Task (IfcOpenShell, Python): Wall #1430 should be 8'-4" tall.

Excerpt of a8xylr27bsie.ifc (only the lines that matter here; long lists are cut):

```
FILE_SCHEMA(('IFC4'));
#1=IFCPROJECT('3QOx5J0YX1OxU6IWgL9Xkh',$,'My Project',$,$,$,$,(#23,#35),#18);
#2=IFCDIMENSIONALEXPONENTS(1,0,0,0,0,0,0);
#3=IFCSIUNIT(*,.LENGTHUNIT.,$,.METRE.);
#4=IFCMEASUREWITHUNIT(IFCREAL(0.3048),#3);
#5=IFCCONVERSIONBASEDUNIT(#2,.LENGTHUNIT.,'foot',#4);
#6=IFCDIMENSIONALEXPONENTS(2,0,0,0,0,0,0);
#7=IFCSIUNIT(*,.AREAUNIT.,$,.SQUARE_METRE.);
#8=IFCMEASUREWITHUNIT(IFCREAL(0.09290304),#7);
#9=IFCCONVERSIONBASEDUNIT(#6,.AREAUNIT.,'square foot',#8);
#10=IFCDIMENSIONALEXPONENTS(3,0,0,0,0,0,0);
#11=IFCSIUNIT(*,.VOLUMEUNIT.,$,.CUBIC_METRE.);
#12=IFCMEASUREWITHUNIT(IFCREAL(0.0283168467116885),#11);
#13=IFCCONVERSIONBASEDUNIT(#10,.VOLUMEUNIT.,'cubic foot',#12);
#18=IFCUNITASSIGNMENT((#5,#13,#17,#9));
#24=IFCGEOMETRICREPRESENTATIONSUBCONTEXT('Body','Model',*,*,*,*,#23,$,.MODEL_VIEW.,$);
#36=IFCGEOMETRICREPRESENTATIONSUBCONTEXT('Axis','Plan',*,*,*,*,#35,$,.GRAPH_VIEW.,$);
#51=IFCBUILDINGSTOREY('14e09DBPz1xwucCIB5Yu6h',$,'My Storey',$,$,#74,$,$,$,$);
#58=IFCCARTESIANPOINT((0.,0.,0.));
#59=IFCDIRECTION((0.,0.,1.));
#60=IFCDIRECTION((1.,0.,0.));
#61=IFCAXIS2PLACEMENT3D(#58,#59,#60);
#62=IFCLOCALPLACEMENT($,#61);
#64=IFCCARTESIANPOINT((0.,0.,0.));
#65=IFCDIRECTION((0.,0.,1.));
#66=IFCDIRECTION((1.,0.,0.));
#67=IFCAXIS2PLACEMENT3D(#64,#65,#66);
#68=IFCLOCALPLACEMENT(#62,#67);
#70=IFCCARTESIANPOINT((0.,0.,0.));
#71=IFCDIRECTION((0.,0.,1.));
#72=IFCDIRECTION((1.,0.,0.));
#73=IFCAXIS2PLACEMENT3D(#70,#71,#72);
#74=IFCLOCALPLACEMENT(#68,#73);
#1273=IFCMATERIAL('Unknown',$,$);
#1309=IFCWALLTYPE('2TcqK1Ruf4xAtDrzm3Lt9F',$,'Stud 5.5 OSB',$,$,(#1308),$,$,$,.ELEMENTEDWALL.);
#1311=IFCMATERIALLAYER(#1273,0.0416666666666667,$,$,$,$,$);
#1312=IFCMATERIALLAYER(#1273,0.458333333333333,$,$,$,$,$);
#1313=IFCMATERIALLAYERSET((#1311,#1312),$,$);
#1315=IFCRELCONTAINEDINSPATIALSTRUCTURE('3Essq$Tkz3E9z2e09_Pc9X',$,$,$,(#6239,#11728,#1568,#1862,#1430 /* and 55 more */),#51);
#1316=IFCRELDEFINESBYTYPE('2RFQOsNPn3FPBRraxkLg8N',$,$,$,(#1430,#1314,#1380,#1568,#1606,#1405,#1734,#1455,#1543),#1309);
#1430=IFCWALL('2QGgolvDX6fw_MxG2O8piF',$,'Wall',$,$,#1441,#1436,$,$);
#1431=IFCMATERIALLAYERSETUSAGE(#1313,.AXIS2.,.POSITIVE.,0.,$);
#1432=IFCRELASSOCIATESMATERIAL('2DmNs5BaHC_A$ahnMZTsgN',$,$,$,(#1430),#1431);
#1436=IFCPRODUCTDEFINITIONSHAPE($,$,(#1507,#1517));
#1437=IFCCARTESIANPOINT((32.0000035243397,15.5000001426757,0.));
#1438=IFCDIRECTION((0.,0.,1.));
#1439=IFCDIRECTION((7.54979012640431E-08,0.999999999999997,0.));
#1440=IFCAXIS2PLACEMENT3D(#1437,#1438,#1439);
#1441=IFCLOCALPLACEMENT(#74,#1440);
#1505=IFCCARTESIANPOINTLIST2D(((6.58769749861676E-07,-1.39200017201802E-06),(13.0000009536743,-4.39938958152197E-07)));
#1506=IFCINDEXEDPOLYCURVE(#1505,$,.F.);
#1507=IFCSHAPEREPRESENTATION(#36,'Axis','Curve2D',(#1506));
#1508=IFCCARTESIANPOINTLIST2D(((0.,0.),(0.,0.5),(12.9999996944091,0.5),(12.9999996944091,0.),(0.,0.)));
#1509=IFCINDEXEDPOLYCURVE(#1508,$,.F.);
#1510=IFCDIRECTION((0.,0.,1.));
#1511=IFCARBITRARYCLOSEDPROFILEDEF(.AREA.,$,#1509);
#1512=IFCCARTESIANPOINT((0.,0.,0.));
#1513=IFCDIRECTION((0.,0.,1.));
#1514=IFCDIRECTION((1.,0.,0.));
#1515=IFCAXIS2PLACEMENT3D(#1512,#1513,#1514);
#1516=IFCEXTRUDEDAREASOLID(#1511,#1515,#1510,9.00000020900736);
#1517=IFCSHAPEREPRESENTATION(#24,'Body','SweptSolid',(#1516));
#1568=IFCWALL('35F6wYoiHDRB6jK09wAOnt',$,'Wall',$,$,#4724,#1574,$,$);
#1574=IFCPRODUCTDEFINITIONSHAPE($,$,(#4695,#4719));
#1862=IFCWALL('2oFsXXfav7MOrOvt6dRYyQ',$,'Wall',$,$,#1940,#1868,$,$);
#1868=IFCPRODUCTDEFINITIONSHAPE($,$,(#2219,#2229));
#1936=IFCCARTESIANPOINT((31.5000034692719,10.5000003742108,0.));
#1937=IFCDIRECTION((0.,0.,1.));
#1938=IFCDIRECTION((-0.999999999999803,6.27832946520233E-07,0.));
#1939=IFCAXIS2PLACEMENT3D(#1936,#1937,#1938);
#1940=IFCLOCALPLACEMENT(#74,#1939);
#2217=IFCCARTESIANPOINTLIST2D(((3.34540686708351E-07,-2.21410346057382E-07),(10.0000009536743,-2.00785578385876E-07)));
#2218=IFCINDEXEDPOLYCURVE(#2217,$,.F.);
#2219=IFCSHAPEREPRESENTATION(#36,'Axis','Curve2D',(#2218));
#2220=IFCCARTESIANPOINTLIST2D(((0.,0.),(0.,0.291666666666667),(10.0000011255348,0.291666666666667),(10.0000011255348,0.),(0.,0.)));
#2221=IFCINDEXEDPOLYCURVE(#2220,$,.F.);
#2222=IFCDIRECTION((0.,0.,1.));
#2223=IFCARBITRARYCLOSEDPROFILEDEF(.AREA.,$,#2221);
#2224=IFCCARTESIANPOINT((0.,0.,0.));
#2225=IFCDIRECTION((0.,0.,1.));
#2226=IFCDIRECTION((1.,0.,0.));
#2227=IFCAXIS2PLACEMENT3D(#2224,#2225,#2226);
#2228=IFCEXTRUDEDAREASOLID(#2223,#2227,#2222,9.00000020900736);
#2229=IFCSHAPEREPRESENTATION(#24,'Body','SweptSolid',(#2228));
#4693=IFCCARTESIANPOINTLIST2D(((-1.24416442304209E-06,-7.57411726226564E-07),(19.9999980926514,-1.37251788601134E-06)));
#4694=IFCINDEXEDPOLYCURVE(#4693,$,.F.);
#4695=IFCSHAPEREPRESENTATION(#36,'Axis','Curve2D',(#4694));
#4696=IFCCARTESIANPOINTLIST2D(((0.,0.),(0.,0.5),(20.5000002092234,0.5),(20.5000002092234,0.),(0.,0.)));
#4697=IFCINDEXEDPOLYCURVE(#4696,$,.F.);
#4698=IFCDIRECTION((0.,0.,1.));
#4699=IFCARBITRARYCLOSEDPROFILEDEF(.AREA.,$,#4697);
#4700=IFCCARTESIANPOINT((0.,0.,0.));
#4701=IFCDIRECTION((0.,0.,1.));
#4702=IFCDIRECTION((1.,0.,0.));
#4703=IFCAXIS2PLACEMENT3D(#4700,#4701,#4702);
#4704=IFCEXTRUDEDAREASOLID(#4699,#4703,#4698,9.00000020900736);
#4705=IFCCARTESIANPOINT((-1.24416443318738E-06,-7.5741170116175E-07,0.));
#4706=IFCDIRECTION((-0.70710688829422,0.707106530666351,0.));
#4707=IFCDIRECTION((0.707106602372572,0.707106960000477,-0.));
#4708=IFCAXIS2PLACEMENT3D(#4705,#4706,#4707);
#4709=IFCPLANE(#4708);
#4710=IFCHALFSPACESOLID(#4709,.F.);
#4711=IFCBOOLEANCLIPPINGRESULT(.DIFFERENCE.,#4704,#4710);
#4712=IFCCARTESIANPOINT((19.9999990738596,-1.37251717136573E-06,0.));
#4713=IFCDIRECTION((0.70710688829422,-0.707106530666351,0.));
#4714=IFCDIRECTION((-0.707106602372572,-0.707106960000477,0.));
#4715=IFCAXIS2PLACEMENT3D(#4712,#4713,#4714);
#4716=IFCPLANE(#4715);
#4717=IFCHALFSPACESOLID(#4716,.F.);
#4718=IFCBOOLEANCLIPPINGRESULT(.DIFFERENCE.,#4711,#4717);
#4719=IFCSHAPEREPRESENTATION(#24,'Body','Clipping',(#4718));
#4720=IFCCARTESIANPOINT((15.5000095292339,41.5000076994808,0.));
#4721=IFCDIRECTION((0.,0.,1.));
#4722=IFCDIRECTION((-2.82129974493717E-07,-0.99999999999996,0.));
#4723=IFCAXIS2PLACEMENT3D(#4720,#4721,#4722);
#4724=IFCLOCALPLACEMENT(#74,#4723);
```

```python
import ifcopenshell
import ifcopenshell.geom
import ifcopenshell.util.representation
import ifcopenshell.util.shape
import ifcopenshell.util.unit

model = ifcopenshell.open("a8xylr27bsie.ifc")
unit_scale = ifcopenshell.util.unit.calculate_unit_scale(model)
settings = ifcopenshell.geom.settings()


def volume(element):
    """Net volume in cubic metres, openings subtracted."""
    shape = ifcopenshell.geom.create_shape(settings, element)
    return ifcopenshell.util.shape.get_volume(shape.geometry)


wall = model.by_id(1430)
before = volume(wall)

body = ifcopenshell.util.representation.get_representation(wall, "Model", "Body")
solid = body.Items[0]
old_height = solid.Depth
solid.Depth = 100 * 0.0254 / unit_scale
after = volume(wall)

print(f"height {old_height:g} -> {solid.Depth:g}, volume {before:.3f} -> {after:.3f} m3")

model.write("a8xylr27bsie_v2.ifc")
```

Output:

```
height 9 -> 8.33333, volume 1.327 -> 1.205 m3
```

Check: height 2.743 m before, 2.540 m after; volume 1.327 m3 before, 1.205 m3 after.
